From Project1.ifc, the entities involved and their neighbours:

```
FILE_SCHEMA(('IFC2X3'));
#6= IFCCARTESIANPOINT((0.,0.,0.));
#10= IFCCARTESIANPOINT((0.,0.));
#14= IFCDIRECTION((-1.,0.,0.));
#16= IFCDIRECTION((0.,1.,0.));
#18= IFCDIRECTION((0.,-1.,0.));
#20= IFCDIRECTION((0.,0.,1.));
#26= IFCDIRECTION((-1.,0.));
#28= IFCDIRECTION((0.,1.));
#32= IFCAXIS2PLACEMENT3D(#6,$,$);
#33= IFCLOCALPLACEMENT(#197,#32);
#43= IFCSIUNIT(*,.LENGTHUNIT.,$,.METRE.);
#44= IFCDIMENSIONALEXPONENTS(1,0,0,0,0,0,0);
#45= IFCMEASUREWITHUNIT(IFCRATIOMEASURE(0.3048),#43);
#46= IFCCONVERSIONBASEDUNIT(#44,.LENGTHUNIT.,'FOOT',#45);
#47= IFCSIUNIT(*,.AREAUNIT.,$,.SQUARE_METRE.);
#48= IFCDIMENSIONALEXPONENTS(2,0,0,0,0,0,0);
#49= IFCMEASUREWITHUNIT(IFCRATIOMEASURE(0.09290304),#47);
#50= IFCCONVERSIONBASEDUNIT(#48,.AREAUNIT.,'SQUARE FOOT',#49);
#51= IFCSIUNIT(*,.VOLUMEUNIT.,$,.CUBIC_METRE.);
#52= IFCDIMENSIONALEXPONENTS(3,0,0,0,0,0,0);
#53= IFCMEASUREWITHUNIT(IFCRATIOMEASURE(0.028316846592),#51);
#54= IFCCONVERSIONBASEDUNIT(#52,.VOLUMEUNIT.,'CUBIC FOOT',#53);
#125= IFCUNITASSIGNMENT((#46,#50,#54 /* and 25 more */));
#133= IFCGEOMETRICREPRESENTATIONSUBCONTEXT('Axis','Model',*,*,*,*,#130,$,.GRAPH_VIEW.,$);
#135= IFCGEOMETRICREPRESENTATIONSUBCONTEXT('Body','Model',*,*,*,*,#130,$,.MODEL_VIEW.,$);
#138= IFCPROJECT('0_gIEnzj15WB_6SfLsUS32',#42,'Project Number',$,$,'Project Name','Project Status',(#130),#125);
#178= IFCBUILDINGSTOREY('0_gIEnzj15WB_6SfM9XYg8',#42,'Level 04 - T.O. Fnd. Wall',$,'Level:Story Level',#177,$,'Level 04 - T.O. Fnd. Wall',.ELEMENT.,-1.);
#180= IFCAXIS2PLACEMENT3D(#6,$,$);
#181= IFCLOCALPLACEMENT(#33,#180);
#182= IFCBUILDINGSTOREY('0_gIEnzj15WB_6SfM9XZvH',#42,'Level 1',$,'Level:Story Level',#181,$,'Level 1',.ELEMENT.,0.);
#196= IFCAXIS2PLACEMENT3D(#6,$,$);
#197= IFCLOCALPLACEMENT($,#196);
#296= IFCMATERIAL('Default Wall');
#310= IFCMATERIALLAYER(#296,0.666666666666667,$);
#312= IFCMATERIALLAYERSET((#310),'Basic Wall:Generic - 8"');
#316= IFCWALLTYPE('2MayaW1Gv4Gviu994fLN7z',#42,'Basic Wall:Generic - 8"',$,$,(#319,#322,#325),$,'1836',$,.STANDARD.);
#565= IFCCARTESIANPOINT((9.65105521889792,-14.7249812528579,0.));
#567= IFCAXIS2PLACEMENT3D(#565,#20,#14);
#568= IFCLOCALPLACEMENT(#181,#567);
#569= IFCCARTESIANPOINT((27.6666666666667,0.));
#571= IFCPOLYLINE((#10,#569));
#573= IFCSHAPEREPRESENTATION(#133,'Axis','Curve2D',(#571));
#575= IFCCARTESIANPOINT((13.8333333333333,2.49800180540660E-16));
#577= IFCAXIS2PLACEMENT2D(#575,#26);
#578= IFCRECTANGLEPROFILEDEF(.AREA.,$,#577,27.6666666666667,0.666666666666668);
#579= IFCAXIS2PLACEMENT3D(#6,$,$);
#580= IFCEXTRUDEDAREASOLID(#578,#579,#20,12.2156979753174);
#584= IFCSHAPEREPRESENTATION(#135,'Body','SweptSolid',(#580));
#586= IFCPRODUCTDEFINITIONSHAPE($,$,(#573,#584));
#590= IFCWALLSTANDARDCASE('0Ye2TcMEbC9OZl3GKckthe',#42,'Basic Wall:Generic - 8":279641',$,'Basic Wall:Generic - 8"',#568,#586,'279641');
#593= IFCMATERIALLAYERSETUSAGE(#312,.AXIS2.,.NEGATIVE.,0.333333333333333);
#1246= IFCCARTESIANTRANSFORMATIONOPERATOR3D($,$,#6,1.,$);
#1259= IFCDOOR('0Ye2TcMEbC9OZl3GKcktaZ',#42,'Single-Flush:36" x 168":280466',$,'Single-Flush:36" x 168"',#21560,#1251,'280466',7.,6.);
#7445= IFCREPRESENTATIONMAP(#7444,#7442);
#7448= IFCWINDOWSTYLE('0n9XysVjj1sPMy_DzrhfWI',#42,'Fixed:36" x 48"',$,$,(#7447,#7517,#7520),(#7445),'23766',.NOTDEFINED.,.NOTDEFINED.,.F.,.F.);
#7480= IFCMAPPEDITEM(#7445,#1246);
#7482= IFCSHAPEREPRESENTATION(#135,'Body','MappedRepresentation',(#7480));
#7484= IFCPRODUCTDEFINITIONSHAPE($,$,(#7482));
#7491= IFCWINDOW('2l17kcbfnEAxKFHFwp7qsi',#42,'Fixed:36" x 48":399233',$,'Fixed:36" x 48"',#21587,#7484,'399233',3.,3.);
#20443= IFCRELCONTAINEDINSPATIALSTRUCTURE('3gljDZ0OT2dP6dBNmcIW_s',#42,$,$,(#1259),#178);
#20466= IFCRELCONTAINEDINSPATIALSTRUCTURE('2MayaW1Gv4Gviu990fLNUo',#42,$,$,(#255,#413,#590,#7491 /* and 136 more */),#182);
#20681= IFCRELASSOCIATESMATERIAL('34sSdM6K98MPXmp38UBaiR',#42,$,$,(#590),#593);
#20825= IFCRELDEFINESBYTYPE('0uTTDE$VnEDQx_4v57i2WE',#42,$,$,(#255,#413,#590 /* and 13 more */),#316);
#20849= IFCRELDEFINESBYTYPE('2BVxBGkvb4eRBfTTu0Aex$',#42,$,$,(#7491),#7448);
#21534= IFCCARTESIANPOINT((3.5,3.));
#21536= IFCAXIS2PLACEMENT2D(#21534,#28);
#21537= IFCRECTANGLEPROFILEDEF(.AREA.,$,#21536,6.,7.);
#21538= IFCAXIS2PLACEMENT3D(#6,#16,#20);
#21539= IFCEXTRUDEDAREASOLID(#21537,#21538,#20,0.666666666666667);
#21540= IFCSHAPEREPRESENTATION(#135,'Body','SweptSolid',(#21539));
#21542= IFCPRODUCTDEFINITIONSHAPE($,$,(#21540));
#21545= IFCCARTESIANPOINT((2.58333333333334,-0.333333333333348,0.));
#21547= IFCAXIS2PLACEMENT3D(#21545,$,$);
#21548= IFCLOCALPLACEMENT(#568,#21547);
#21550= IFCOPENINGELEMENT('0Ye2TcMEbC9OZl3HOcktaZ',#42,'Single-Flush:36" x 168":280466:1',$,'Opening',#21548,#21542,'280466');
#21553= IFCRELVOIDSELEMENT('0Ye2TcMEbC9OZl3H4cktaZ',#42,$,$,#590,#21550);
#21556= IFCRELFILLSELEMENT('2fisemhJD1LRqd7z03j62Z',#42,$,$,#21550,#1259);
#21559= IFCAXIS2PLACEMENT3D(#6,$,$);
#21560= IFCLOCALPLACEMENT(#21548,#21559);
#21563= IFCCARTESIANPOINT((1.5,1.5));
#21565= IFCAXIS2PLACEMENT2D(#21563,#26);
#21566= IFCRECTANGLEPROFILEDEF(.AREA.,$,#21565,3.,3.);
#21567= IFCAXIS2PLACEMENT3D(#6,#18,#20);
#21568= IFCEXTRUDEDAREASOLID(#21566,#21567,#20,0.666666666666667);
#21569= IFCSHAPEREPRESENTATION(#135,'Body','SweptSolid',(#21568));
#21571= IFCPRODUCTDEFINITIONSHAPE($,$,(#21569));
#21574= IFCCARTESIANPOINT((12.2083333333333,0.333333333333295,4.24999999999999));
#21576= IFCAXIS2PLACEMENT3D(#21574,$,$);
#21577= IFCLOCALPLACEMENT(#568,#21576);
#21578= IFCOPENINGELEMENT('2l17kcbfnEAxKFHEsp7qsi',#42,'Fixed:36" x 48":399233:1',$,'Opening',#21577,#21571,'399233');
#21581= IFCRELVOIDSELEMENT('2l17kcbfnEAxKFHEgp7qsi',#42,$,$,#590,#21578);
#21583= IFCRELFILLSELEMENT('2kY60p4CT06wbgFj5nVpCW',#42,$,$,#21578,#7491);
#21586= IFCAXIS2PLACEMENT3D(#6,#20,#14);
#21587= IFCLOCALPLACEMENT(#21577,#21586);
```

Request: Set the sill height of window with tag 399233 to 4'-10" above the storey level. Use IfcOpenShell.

```python
import numpy as np
import ifcopenshell
import ifcopenshell.api.geometry
import ifcopenshell.geom
import ifcopenshell.util.element
import ifcopenshell.util.placement
import ifcopenshell.util.shape
import ifcopenshell.util.unit

model = ifcopenshell.open("Project1.ifc")
unit_scale = ifcopenshell.util.unit.calculate_unit_scale(model)

window = model.by_id(7491)
opening = window.FillsVoids[0].RelatingOpeningElement
storey = ifcopenshell.util.element.get_container(window, ifc_class="IfcBuildingStorey")
level = ifcopenshell.util.placement.get_local_placement(storey.ObjectPlacement)[2, 3]

# The opening's origin need not be at the sill, so measure its lowest point.
shape = ifcopenshell.geom.create_shape(ifcopenshell.geom.settings(), opening)
bottom = ifcopenshell.util.shape.get_shape_bottom_elevation(shape, shape.geometry) / unit_scale
dz = level + 58 * 0.0254 / unit_scale - bottom

shift = np.array([0.0, 0.0, dz])
# The window is placed relative to its opening, so it follows when the opening moves.
matrix = ifcopenshell.util.placement.get_local_placement(opening.ObjectPlacement)
matrix[:3, 3] += shift
ifcopenshell.api.geometry.edit_object_placement(
    model, product=opening, matrix=matrix, is_si=False, should_transform_children=True
)

print(f"moved by {dz * unit_scale:+.3f} m")

model.write("Project1-out.ifc")
```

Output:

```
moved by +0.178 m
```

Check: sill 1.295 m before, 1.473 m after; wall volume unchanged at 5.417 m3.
